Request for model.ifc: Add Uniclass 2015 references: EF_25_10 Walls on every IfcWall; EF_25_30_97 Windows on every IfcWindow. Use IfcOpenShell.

First a look at what the model holds.

```python
import ifcopenshell

model = ifcopenshell.open("model.ifc")
print(model.schema)
print("classifications:", [c.Name for c in model.by_type("IfcClassification")])
for ifc_class in ("IfcDoor", "IfcRoof", "IfcStair", "IfcWall", "IfcWindow"):
    print(ifc_class, len(model.by_type(ifc_class)))
```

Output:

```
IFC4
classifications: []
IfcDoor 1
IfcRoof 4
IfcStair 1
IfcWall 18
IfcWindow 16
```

```python
import ifcopenshell
import ifcopenshell.api.classification

model = ifcopenshell.open("model.ifc")

system = ifcopenshell.api.classification.add_classification(model, classification="Uniclass 2015")

codes = {
    "IfcWall": ("EF_25_10", "Walls"),
    "IfcWindow": ("EF_25_30_97", "Windows"),
}
for ifc_class, (code, name) in codes.items():
    products = model.by_type(ifc_class)
    ifcopenshell.api.classification.add_reference(
        model, products=products, classification=system, identification=code, name=name
    )
    print(code, len(products))

model.write("model-out.ifc")
```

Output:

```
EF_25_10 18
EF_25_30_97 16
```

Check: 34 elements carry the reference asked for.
